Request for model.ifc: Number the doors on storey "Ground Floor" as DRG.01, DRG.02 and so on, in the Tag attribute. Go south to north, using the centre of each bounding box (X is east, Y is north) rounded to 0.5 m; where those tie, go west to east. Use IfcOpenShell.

First a look at what the model holds.

```python
import ifcopenshell
import ifcopenshell.util.element
import ifcopenshell.util.placement

model = ifcopenshell.open("model.ifc")
print(model.schema)
storey = next(s for s in model.by_type("IfcBuildingStorey") if s.Name == "Ground Floor")
doors = [e for e in ifcopenshell.util.element.get_decomposition(storey) if e.is_a("IfcDoor")]
for e in sorted(doors, key=lambda e: e.id()):
    origin = ifcopenshell.util.placement.get_local_placement(e.ObjectPlacement)[:3, 3]
    print(e.id(), e.Tag, e.Name, origin.round(2) + 0.0, sep=" | ")
```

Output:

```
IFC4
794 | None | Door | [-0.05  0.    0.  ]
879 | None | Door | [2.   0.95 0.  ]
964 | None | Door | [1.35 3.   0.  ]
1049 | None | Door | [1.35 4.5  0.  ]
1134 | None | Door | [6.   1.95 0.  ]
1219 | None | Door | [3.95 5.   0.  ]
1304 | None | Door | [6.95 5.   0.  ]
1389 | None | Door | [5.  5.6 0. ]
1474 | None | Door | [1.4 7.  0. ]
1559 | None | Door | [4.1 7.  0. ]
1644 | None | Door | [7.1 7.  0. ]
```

```python
import ifcopenshell
import ifcopenshell.geom
import ifcopenshell.util.element
import ifcopenshell.util.shape

model = ifcopenshell.open("model.ifc")
settings = ifcopenshell.geom.settings()
settings.set("use-world-coords", True)


def centre(element):
    shape = ifcopenshell.geom.create_shape(settings, element)
    return ifcopenshell.util.shape.get_bbox_centroid(shape.geometry)


storey = next(s for s in model.by_type("IfcBuildingStorey") if s.Name == "Ground Floor")
doors = [e for e in ifcopenshell.util.element.get_decomposition(storey) if e.is_a("IfcDoor")]

# Insertion points can sit at a corner or the storey origin, so sort by the geometry (in metres).
centres = {e: centre(e) for e in doors}
doors.sort(key=lambda e: (round(centres[e][1] / 0.5), centres[e][0]))

for i, e in enumerate(doors, start=1):
    number = f"DRG.{i:02d}"
    e.Tag = number
    print(e.id(), number)

model.write("model_updated.ifc")
```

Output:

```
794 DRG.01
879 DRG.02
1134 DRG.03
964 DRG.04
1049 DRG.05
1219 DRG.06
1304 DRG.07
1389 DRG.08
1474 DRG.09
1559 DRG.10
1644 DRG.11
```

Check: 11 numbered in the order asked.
